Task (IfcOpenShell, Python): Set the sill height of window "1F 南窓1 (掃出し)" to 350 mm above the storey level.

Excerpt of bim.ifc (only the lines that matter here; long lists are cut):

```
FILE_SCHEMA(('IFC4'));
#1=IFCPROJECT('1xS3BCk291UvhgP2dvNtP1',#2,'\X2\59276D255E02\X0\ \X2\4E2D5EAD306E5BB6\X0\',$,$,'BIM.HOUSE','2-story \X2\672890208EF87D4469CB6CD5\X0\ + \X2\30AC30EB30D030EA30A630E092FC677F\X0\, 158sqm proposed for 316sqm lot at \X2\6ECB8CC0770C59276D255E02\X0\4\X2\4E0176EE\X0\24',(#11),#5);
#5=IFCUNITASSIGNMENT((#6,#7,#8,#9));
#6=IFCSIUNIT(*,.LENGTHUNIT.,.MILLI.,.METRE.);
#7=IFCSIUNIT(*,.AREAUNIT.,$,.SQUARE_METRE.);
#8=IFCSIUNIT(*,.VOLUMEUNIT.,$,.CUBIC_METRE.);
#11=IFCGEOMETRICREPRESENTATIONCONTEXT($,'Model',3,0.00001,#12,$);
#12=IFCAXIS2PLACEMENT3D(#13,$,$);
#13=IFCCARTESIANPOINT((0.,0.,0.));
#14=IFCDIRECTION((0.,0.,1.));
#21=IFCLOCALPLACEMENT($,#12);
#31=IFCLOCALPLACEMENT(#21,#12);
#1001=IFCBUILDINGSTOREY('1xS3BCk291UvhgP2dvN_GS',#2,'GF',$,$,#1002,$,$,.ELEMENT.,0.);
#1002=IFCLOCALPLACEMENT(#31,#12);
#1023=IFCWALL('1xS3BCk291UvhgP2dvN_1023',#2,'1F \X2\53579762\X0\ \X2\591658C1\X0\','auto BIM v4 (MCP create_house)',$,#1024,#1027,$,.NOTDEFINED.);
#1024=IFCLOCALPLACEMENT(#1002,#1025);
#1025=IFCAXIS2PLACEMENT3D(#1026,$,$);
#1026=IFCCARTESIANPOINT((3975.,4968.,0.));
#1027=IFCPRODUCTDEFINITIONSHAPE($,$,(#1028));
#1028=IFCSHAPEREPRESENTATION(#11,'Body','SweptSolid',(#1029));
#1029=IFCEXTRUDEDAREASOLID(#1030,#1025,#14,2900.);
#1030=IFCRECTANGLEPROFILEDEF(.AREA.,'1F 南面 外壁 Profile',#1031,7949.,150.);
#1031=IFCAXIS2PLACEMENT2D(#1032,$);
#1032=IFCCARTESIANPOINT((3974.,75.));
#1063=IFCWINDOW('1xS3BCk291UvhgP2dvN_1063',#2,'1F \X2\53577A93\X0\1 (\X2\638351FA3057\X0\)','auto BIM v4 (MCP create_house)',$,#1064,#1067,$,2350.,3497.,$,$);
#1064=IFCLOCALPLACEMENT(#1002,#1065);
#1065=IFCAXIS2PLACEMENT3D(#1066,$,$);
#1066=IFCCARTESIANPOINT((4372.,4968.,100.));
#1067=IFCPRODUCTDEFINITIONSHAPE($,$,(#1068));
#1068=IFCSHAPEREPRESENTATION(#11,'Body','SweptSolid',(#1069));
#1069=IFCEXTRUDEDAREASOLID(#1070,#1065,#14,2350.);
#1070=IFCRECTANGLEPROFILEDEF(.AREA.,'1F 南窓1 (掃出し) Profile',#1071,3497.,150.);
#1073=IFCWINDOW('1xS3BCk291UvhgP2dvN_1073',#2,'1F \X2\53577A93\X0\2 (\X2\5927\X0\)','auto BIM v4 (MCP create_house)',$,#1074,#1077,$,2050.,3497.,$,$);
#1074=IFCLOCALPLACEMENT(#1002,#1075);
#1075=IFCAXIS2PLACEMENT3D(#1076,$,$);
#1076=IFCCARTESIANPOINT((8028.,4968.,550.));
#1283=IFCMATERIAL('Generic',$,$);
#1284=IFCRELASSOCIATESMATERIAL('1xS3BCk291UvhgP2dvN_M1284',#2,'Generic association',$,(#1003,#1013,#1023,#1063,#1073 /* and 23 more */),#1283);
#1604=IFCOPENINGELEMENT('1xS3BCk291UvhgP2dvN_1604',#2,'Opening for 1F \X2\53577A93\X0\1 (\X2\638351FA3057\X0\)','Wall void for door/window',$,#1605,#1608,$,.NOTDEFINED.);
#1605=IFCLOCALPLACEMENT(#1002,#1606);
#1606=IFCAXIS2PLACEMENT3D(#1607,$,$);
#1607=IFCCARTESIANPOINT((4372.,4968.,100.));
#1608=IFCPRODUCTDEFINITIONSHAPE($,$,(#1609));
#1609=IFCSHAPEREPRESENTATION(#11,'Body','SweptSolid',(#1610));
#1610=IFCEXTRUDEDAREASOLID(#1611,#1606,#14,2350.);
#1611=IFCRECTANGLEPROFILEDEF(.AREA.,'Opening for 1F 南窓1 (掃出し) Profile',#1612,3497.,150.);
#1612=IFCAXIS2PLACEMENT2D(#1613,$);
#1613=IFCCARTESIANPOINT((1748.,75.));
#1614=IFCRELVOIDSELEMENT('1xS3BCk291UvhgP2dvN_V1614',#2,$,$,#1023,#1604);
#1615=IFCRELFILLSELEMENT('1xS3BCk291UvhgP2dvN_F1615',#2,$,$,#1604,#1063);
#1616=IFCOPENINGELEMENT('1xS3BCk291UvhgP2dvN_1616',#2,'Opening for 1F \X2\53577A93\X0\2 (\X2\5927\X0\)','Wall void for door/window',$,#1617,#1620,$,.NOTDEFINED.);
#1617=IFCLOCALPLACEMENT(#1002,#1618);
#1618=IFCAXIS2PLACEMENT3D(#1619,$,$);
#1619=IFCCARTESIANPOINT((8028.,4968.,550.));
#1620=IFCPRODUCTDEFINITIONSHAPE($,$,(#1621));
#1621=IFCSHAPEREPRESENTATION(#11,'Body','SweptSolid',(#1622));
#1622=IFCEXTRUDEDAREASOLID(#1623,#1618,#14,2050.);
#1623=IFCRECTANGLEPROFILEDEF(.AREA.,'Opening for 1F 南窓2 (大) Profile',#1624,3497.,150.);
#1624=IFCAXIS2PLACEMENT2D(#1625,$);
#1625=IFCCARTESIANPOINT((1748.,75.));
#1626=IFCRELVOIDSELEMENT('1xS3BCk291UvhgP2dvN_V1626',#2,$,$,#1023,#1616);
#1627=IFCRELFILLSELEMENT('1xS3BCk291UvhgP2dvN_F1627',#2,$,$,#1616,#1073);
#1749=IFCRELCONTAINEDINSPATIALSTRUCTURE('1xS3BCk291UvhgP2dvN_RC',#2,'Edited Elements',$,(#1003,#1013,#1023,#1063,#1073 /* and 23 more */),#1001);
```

```python
import numpy as np
import ifcopenshell
import ifcopenshell.api.geometry
import ifcopenshell.geom
import ifcopenshell.util.element
import ifcopenshell.util.placement
import ifcopenshell.util.shape
import ifcopenshell.util.unit

model = ifcopenshell.open("bim.ifc")
unit_scale = ifcopenshell.util.unit.calculate_unit_scale(model)

window = model.by_guid("1xS3BCk291UvhgP2dvN_1063")
opening = window.FillsVoids[0].RelatingOpeningElement
storey = ifcopenshell.util.element.get_container(window, ifc_class="IfcBuildingStorey")
level = ifcopenshell.util.placement.get_local_placement(storey.ObjectPlacement)[2, 3]

# The opening's origin need not be at the sill, so measure its lowest point.
shape = ifcopenshell.geom.create_shape(ifcopenshell.geom.settings(), opening)
bottom = ifcopenshell.util.shape.get_shape_bottom_elevation(shape, shape.geometry) / unit_scale
dz = level + 0.35 / unit_scale - bottom

shift = np.array([0.0, 0.0, dz])
# The window is not placed relative to its opening, so move both.
for product in (opening, window):
    matrix = ifcopenshell.util.placement.get_local_placement(product.ObjectPlacement)
    matrix[:3, 3] += shift
    ifcopenshell.api.geometry.edit_object_placement(model, product=product, matrix=matrix, is_si=False)

print(f"moved by {dz * unit_scale:+.3f} m")

model.write("bim-out.ifc")
```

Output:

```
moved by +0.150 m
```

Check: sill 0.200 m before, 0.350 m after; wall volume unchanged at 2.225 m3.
